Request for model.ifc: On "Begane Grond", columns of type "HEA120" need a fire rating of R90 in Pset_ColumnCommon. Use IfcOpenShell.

First a look at what the model holds.

```python
import ifcopenshell
import ifcopenshell.util.element

model = ifcopenshell.open("model.ifc")
print(model.schema)
storey = next(s for s in model.by_type("IfcBuildingStorey") if s.Name == "Begane Grond")
columns = [e for e in ifcopenshell.util.element.get_decomposition(storey) if e.is_a("IfcColumn")]
seen = {}
for e in columns:
    element_type = ifcopenshell.util.element.get_type(e)
    key = (element_type.Name if element_type != e and element_type else None, ifcopenshell.util.element.get_pset(e, "Pset_ColumnCommon", "FireRating"))
    seen[key] = seen.get(key, 0) + 1
for (name, value), count in sorted(seen.items(), key=str):
    print(count, "x", name, "|", value)
```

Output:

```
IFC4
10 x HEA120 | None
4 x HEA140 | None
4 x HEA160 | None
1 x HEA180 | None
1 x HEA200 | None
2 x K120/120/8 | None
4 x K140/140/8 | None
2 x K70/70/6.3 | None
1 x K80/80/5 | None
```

```python
import ifcopenshell
import ifcopenshell.api.pset
import ifcopenshell.util.element

model = ifcopenshell.open("model.ifc")

storey = next(s for s in model.by_type("IfcBuildingStorey") if s.Name == "Begane Grond")
columns = [e for e in ifcopenshell.util.element.get_decomposition(storey) if e.is_a("IfcColumn")]

count = 0
for e in columns:
    element_type = ifcopenshell.util.element.get_type(e)
    if element_type in (None, e) or element_type.Name != "HEA120":
        continue
    # add_pset returns the element's existing set when there is one.
    pset = ifcopenshell.api.pset.add_pset(model, product=e, name="Pset_ColumnCommon")
    ifcopenshell.api.pset.edit_pset(model, pset=pset, properties={"FireRating": "R90"})
    count += 1

print(count, "columns updated")

model.write("model_v2.ifc")
```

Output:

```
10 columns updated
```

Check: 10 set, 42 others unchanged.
